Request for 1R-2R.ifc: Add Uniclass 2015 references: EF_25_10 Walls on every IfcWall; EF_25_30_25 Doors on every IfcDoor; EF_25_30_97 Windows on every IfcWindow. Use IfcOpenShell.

First a look at what the model holds.

```python
import ifcopenshell

model = ifcopenshell.open("1R-2R.ifc")
print(model.schema)
print("classifications:", [c.Name for c in model.by_type("IfcClassification")])
for ifc_class in ("IfcDoor", "IfcRoof", "IfcStair", "IfcWall", "IfcWindow"):
    print(ifc_class, len(model.by_type(ifc_class)))
```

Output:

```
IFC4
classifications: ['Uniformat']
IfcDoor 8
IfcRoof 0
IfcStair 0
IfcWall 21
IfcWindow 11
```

```python
import ifcopenshell
import ifcopenshell.api.classification

model = ifcopenshell.open("1R-2R.ifc")

system = ifcopenshell.api.classification.add_classification(model, classification="Uniclass 2015")

codes = {
    "IfcWall": ("EF_25_10", "Walls"),
    "IfcDoor": ("EF_25_30_25", "Doors"),
    "IfcWindow": ("EF_25_30_97", "Windows"),
}
for ifc_class, (code, name) in codes.items():
    products = model.by_type(ifc_class)
    ifcopenshell.api.classification.add_reference(
        model, products=products, classification=system, identification=code, name=name
    )
    print(code, len(products))

model.write("1R-2R_v2.ifc")
```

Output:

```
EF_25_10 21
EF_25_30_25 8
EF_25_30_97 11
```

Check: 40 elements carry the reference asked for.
